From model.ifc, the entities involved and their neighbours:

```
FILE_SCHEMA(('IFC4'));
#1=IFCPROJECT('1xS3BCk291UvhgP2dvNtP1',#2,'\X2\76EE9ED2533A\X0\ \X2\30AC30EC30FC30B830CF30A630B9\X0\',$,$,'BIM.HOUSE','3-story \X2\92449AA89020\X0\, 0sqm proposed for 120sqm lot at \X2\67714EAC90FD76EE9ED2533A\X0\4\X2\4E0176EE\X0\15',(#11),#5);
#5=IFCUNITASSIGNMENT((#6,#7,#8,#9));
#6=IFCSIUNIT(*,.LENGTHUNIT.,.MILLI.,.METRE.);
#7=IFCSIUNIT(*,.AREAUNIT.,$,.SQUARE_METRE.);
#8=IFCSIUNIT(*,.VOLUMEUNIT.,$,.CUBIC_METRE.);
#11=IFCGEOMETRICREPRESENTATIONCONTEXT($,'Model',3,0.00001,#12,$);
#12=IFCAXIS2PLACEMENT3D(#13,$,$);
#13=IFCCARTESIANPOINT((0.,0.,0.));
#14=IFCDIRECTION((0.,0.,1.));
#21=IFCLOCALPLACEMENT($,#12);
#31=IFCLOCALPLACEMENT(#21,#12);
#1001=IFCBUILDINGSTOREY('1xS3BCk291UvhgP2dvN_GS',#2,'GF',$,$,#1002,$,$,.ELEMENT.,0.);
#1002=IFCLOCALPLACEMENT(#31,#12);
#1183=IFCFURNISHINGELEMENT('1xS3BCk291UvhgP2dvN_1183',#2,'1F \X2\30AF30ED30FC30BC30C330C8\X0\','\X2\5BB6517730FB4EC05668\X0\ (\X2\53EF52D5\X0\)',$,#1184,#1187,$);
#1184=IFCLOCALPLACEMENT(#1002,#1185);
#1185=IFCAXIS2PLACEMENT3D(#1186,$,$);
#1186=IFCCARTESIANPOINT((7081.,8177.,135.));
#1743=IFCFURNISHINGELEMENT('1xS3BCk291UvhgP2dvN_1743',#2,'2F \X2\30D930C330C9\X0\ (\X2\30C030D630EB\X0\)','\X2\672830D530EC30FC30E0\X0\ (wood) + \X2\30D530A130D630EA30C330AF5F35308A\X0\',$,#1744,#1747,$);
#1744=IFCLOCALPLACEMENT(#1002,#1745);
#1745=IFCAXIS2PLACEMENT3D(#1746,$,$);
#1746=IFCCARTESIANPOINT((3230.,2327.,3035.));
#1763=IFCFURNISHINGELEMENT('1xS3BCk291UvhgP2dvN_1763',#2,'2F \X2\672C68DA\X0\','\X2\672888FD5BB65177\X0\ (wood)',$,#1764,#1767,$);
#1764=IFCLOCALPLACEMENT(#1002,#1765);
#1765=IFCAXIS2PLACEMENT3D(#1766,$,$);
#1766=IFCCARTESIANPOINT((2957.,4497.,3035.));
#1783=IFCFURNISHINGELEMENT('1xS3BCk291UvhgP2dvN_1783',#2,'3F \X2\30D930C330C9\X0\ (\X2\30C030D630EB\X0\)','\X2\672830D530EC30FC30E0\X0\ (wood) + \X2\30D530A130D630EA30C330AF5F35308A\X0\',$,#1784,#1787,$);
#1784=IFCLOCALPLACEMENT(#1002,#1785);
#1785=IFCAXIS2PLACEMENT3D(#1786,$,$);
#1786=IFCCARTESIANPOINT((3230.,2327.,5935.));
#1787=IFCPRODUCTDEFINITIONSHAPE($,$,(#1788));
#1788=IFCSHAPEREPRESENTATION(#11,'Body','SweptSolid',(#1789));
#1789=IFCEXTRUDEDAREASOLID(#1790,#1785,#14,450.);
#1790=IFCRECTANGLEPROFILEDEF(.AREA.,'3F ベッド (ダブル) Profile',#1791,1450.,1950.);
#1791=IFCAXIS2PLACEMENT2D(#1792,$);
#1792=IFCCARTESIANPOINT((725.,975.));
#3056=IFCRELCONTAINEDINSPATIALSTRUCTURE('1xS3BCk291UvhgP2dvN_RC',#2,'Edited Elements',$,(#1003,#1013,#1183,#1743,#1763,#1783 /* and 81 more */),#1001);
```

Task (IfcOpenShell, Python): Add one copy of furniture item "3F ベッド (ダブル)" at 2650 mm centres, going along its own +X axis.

```python
import ifcopenshell
import ifcopenshell.api.geometry
import ifcopenshell.api.root
import ifcopenshell.util.element
import ifcopenshell.util.placement
import ifcopenshell.util.unit

model = ifcopenshell.open("model.ifc")
unit_scale = ifcopenshell.util.unit.calculate_unit_scale(model)


def reuse_history(source, copy):
    """copy_class also copies each property set's owner history, people and application; keep the originals."""
    for rel in copy.IsDefinedBy:
        if rel.is_a("IfcRelDefinesByProperties") and (history := rel.RelatingPropertyDefinition.OwnerHistory):
            rel.RelatingPropertyDefinition.OwnerHistory = source.OwnerHistory
            ifcopenshell.util.element.remove_deep2(model, history)


source = model.by_id(1783)
base = ifcopenshell.util.placement.get_local_placement(source.ObjectPlacement)
step = base[:3, 0] * 2.65 / unit_scale

for i in range(1, 2):
    copy = ifcopenshell.api.root.copy_class(model, product=source)
    copy.Representation = ifcopenshell.util.element.copy_deep(
        model, source.Representation, exclude=["IfcGeometricRepresentationContext", "IfcRepresentationMap"]
    )
    reuse_history(source, copy)
    matrix = base.copy()
    matrix[:3, 3] += i * step
    print("added at", matrix[:3, 3].round(3) + 0.0)
    ifcopenshell.api.geometry.edit_object_placement(model, product=copy, matrix=matrix, is_si=False)

model.write("model_edited.ifc")
```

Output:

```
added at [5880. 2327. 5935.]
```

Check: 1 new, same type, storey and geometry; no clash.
